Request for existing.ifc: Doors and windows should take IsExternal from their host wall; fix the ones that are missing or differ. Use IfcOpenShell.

First a look at what the model holds.

```python
import ifcopenshell
import ifcopenshell.util.element

model = ifcopenshell.open("existing.ifc")
print(model.schema)
seen = {}
for e in model.by_type("IfcDoor") + model.by_type("IfcWindow"):
    if not e.FillsVoids:
        continue
    host = e.FillsVoids[0].RelatingOpeningElement.VoidsElements[0].RelatingBuildingElement
    own = ifcopenshell.util.element.get_pset(e, f"Pset_{e.is_a()[3:].removesuffix('StandardCase')}Common", "IsExternal")
    wall = ifcopenshell.util.element.get_pset(host, "Pset_WallCommon", "IsExternal")
    seen[e.is_a(), own, wall] = seen.get((e.is_a(), own, wall), 0) + 1
for (cls, own, wall), count in sorted(seen.items(), key=str):
    print(count, cls, "IsExternal:", own, "| host wall:", wall)
```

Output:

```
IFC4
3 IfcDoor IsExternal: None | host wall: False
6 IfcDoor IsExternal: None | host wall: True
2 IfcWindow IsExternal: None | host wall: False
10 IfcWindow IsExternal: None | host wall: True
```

```python
import ifcopenshell
import ifcopenshell.api.pset
import ifcopenshell.util.element

model = ifcopenshell.open("existing.ifc")

count = 0
for ifc_class, pset_name in (("IfcDoor", "Pset_DoorCommon"), ("IfcWindow", "Pset_WindowCommon")):
    for e in model.by_type(ifc_class):
        if not e.FillsVoids:
            continue
        host = e.FillsVoids[0].RelatingOpeningElement.VoidsElements[0].RelatingBuildingElement
        external = ifcopenshell.util.element.get_pset(host, "Pset_WallCommon", "IsExternal")
        if external is None or ifcopenshell.util.element.get_pset(e, pset_name, "IsExternal") == external:
            continue
        pset = ifcopenshell.api.pset.add_pset(model, product=e, name=pset_name)
        ifcopenshell.api.pset.edit_pset(model, pset=pset, properties={"IsExternal": external})
        count += 1

print(count, "updated")

model.write("existing_rev.ifc")
```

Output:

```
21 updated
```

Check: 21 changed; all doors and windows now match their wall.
